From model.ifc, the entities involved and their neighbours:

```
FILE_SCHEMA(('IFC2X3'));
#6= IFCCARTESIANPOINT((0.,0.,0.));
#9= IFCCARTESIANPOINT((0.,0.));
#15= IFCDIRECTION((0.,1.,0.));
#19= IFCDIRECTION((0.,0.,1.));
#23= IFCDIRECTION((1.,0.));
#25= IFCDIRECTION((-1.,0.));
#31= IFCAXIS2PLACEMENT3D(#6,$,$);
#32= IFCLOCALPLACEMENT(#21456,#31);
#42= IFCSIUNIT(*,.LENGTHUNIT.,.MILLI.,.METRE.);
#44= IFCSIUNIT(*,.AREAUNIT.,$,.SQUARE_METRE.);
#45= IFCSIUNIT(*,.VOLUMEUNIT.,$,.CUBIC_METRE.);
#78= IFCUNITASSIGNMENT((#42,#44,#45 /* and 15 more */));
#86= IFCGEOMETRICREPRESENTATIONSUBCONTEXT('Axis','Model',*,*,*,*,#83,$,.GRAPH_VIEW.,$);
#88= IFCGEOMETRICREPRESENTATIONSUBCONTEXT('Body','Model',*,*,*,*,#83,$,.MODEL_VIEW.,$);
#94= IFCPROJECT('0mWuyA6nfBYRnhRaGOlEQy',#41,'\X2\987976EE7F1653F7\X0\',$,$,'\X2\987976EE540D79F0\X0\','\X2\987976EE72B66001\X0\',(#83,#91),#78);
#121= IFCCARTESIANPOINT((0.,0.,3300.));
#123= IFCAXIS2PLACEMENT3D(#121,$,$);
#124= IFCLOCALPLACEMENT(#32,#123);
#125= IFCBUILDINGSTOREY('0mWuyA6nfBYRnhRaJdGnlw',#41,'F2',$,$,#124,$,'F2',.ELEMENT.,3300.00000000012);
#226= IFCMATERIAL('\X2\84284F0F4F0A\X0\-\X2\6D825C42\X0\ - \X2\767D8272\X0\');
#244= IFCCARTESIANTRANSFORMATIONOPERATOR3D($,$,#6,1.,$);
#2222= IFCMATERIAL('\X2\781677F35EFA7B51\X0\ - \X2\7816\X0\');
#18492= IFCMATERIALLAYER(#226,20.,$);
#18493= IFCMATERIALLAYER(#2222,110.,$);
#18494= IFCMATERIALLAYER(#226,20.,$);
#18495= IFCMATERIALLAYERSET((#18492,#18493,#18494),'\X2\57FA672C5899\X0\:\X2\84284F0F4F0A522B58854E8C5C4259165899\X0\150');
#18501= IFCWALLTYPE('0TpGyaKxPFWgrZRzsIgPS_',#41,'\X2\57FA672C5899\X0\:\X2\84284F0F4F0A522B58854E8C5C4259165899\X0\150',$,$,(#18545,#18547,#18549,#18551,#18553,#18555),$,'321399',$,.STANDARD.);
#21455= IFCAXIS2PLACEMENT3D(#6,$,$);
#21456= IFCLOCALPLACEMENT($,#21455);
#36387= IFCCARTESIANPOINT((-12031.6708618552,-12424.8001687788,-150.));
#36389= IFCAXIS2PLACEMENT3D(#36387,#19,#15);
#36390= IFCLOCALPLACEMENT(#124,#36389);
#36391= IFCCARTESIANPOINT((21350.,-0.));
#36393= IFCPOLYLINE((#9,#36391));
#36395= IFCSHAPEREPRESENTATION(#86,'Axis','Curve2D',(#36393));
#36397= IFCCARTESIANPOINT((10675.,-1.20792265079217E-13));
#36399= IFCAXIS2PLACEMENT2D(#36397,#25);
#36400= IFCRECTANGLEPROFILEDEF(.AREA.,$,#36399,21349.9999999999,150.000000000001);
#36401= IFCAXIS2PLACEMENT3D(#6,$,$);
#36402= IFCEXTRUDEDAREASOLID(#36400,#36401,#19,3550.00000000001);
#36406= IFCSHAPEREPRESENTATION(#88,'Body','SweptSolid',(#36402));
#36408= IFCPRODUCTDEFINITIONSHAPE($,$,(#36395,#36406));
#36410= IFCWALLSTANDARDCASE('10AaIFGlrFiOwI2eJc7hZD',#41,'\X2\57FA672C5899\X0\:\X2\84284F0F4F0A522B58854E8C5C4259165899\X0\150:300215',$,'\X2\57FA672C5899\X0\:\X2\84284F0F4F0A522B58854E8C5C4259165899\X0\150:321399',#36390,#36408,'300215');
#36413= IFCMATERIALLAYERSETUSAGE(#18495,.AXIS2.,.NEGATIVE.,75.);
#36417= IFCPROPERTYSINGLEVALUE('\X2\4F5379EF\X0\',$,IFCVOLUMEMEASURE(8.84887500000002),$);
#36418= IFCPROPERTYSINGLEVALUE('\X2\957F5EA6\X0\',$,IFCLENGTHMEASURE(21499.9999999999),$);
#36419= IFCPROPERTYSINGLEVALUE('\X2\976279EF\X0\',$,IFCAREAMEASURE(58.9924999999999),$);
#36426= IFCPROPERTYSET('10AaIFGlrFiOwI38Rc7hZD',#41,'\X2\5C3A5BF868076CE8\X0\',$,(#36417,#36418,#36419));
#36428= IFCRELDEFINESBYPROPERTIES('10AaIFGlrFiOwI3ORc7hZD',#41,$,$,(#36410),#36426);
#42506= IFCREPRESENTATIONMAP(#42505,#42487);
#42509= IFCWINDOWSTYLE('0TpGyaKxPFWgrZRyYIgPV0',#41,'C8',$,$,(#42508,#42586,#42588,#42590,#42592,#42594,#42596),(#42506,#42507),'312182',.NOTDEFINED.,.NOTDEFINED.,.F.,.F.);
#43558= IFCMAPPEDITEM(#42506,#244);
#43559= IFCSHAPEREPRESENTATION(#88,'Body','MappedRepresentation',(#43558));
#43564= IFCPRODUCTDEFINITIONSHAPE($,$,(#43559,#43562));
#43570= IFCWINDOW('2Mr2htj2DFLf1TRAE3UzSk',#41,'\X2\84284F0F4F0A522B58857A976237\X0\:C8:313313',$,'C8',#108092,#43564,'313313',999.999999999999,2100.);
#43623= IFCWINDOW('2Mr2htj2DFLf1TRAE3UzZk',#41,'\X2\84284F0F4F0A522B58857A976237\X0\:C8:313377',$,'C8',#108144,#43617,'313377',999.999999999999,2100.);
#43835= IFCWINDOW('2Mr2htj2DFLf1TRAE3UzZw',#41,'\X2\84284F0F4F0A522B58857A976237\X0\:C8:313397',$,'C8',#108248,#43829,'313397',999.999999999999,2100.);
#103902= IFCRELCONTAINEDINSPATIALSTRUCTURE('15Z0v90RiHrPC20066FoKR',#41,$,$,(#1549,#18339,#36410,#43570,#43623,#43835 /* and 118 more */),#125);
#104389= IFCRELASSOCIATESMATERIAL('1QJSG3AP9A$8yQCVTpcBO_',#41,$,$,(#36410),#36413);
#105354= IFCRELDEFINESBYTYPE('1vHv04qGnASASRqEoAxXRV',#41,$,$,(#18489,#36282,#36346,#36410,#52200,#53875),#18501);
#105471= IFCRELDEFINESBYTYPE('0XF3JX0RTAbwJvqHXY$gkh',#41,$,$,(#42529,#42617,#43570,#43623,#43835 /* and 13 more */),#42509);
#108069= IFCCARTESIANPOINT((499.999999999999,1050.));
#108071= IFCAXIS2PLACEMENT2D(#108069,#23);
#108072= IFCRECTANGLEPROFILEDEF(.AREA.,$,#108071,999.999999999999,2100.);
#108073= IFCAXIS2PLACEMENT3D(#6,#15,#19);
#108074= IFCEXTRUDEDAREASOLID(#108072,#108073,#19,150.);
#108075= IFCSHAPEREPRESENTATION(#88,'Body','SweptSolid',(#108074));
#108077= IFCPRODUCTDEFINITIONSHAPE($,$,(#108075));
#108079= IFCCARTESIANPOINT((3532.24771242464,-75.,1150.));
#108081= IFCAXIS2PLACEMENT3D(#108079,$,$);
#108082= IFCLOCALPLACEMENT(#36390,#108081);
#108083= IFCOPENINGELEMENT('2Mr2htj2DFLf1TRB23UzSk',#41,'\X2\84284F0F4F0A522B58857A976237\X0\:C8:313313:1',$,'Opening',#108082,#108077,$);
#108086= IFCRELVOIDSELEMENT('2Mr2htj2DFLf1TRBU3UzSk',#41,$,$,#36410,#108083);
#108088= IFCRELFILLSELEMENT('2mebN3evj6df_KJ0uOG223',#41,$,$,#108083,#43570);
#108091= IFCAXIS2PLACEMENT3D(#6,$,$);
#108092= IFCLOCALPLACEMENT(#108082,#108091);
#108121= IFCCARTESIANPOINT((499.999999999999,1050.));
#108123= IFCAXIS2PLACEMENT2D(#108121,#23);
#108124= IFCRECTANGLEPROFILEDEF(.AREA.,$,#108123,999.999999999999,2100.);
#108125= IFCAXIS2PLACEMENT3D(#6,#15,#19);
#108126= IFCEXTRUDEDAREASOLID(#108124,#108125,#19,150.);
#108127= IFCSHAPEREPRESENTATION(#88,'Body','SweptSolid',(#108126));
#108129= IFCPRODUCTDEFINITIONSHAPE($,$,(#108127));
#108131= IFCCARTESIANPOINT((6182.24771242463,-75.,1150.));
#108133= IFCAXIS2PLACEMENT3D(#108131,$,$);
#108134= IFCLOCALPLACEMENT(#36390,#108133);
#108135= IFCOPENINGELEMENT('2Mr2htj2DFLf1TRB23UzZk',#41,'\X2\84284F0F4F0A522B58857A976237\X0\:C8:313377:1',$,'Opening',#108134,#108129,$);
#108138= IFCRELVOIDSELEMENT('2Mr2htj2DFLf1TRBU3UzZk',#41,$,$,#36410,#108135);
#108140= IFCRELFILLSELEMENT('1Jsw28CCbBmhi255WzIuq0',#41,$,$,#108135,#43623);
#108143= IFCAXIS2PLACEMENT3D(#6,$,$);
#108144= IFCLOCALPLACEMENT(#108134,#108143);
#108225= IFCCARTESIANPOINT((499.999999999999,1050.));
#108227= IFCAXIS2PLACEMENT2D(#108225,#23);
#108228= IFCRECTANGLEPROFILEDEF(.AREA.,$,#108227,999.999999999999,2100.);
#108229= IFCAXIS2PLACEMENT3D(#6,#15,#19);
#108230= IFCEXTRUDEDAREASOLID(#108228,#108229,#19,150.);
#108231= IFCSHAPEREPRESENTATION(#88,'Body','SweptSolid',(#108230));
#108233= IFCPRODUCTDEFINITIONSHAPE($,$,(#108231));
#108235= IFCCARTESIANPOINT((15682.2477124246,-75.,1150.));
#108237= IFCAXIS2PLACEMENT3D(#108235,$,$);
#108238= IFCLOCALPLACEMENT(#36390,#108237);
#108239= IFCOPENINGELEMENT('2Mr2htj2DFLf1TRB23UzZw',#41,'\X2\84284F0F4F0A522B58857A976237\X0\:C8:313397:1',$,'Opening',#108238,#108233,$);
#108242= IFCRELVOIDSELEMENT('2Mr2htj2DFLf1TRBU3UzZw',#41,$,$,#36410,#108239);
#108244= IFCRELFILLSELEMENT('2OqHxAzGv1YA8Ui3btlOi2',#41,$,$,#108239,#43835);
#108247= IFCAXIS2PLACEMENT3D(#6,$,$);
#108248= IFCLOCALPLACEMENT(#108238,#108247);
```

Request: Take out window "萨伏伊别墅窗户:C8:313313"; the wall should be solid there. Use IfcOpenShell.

```python
import ifcopenshell
import ifcopenshell.api.feature
import ifcopenshell.api.pset
import ifcopenshell.api.root
import ifcopenshell.geom
import ifcopenshell.util.element
import ifcopenshell.util.shape
import ifcopenshell.util.unit

model = ifcopenshell.open("model.ifc")
area_scale = ifcopenshell.util.unit.calculate_unit_scale(model, "AREAUNIT")
volume_scale = ifcopenshell.util.unit.calculate_unit_scale(model, "VOLUMEUNIT")
settings = ifcopenshell.geom.settings()


def volume(element):
    """Net volume in cubic metres, openings subtracted."""
    shape = ifcopenshell.geom.create_shape(settings, element)
    return ifcopenshell.util.shape.get_volume(shape.geometry)


window = model.by_id(43570)
opening = window.FillsVoids[0].RelatingOpeningElement
wall = opening.VoidsElements[0].RelatingBuildingElement
before = volume(wall)

ifcopenshell.api.root.remove_product(model, product=window)
ifcopenshell.api.feature.remove_feature(model, feature=opening)

after = volume(wall)
thickness = 0.15  # wall thickness in metres

# Update the wall's stored quantities.
pset = model.by_id(ifcopenshell.util.element.get_pset(wall, "尺寸标注", should_inherit=False)["id"])
ifcopenshell.api.pset.edit_pset(model, pset=pset, properties={
    "体积": model.create_entity("IfcVolumeMeasure", after / volume_scale),
    "面积": model.create_entity("IfcAreaMeasure", after / thickness / area_scale),
})

print(f"wall volume {before:.3f} -> {after:.3f} m3")

model.write("model-out.ifc")
```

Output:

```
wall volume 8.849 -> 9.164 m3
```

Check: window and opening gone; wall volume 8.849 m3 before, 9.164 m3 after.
